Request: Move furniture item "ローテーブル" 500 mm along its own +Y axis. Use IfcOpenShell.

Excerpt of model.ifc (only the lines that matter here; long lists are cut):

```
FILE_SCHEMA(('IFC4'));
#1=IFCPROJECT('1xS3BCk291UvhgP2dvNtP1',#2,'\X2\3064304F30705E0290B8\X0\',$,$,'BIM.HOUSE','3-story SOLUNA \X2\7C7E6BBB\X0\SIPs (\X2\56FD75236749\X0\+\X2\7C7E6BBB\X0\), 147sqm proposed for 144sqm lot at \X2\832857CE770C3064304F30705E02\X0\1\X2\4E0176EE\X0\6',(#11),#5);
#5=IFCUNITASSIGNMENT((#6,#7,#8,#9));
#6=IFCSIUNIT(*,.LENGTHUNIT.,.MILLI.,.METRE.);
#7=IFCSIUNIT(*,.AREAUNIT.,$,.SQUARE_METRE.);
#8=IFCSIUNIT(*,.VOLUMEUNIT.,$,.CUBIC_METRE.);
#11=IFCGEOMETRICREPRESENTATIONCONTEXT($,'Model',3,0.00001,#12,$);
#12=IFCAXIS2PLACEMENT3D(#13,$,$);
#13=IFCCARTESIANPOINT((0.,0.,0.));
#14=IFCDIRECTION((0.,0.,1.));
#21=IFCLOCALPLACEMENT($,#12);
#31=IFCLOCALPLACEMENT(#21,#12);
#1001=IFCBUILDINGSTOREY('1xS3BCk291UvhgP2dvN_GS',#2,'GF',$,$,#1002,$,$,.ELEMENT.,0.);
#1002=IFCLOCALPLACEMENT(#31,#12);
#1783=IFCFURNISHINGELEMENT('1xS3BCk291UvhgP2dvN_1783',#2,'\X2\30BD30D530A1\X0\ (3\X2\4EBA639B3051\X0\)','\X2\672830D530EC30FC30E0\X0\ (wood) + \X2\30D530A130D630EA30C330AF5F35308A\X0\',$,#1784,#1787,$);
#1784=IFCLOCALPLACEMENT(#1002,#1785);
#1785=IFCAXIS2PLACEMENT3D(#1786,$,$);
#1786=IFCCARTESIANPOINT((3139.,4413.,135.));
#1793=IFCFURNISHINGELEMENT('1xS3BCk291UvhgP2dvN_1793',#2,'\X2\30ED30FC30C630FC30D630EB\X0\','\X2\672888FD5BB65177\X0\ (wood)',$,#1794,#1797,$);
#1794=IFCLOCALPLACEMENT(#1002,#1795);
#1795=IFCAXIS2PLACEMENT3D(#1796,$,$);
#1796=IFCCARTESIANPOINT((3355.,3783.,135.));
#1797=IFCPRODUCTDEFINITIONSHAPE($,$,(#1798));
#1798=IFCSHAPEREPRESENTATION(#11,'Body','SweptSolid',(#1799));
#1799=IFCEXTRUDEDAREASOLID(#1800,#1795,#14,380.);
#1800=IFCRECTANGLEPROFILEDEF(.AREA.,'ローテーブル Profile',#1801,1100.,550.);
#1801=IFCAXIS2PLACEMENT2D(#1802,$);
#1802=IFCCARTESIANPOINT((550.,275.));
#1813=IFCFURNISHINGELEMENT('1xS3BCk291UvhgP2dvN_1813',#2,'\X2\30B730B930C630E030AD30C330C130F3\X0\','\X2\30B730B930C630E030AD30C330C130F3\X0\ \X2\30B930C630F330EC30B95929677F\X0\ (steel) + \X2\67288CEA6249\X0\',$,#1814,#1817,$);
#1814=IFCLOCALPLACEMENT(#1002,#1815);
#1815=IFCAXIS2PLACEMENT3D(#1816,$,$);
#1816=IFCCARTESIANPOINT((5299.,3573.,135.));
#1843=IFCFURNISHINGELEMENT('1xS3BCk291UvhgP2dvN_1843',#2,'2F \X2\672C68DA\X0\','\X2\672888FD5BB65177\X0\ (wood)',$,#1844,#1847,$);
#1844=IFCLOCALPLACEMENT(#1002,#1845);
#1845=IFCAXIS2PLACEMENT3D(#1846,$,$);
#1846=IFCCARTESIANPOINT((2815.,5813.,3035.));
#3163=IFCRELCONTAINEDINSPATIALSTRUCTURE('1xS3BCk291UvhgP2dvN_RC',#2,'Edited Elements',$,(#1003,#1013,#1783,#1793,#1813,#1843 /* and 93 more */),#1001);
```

```python
import ifcopenshell
import ifcopenshell.api.geometry
import ifcopenshell.util.placement
import ifcopenshell.util.unit

model = ifcopenshell.open("model.ifc")
unit_scale = ifcopenshell.util.unit.calculate_unit_scale(model)

item = model.by_guid("1xS3BCk291UvhgP2dvN_1793")
matrix = ifcopenshell.util.placement.get_local_placement(item.ObjectPlacement)
matrix[:3, 3] += matrix[:3, 1] * 0.5 / unit_scale
ifcopenshell.api.geometry.edit_object_placement(model, product=item, matrix=matrix, is_si=False)

print(ifcopenshell.util.placement.get_local_placement(item.ObjectPlacement).round(3) + 0.0)

model.write("model_edited.ifc")
```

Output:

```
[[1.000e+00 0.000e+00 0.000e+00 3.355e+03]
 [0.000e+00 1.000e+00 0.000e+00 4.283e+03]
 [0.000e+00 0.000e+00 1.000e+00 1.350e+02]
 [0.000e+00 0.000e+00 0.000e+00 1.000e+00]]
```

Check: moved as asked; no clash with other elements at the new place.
